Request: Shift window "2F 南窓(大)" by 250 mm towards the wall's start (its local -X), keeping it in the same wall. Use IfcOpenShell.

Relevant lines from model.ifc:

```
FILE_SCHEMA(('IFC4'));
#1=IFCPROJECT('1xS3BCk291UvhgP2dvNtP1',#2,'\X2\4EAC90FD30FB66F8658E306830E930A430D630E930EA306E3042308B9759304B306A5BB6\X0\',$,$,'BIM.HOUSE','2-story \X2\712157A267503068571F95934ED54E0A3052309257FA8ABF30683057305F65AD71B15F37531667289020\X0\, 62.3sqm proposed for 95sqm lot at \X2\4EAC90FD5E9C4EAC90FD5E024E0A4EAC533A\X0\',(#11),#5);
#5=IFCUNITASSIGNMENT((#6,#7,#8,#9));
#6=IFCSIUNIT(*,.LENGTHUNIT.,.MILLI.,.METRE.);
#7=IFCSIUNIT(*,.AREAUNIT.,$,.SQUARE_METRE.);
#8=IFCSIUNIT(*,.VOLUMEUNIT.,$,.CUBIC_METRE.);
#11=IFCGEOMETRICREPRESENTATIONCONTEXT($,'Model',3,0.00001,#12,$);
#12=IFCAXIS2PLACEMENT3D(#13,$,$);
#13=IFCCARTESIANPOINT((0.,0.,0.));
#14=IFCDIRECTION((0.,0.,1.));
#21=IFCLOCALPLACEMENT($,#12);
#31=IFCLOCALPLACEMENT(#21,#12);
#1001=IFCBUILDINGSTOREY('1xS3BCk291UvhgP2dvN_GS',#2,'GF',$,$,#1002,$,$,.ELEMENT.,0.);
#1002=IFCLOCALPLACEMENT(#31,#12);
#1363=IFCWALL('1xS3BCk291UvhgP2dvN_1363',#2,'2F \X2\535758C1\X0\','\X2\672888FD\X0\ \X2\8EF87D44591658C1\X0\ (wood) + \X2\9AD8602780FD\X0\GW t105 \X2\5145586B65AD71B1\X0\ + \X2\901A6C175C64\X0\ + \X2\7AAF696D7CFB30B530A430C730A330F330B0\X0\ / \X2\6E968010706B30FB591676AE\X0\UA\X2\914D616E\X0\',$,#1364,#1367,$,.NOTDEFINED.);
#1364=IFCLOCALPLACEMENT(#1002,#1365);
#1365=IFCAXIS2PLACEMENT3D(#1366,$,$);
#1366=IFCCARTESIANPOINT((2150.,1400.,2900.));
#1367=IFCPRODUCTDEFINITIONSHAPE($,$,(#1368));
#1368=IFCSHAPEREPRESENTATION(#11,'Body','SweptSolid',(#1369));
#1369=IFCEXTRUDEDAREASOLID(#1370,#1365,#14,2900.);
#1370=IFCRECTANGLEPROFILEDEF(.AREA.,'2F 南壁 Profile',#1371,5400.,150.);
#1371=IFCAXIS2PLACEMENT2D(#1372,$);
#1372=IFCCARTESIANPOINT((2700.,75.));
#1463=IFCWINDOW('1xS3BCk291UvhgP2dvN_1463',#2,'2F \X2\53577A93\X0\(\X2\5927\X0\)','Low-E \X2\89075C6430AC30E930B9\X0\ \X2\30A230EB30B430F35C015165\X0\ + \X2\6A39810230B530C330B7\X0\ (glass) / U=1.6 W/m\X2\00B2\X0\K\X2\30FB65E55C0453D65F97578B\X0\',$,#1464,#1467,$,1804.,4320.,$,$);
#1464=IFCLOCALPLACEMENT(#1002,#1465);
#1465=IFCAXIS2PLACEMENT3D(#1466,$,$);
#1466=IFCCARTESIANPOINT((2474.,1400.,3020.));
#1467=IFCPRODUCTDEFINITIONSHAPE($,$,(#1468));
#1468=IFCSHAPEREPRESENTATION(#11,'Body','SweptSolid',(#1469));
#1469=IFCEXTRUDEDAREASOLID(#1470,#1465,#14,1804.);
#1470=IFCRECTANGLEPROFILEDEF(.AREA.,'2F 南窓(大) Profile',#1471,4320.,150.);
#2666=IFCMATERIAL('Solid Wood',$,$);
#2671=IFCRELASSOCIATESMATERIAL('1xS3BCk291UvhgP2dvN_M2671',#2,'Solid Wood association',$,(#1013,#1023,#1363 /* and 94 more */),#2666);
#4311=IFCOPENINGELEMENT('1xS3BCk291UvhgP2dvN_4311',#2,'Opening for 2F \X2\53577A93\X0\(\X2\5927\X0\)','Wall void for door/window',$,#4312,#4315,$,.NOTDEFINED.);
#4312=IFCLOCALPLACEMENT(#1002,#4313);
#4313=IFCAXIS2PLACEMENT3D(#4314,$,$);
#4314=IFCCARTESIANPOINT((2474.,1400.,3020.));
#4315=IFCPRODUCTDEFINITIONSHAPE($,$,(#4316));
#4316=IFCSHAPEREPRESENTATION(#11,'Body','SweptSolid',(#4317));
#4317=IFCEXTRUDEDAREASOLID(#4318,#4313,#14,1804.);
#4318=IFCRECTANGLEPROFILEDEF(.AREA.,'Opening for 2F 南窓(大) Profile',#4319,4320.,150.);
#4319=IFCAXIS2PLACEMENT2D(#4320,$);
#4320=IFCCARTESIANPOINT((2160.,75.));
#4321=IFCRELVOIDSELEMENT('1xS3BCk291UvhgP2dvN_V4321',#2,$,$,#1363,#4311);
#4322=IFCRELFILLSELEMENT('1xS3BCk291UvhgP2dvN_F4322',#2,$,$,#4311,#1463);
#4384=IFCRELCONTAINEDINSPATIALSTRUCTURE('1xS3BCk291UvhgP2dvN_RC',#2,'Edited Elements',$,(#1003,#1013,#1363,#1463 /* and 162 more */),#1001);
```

```python
import ifcopenshell
import ifcopenshell.api.geometry
import ifcopenshell.util.placement

model = ifcopenshell.open("model.ifc")

window = model.by_guid("1xS3BCk291UvhgP2dvN_1463")
opening = window.FillsVoids[0].RelatingOpeningElement
wall = opening.VoidsElements[0].RelatingBuildingElement

wall_matrix = ifcopenshell.util.placement.get_local_placement(wall.ObjectPlacement)
shift = wall_matrix[:3, 0] * -250.0
before = ifcopenshell.util.placement.get_local_placement(window.ObjectPlacement)[:3, 3].copy()

# The window is not placed relative to its opening, so move both.
for product in (opening, window):
    matrix = ifcopenshell.util.placement.get_local_placement(product.ObjectPlacement)
    matrix[:3, 3] += shift
    ifcopenshell.api.geometry.edit_object_placement(model, product=product, matrix=matrix, is_si=False)

after = ifcopenshell.util.placement.get_local_placement(window.ObjectPlacement)[:3, 3]
print("window moved by", (after - before).round(3) + 0.0)

model.write("model_v2.ifc")
```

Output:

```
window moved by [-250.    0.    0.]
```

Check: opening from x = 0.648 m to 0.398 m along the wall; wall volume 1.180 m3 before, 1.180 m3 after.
